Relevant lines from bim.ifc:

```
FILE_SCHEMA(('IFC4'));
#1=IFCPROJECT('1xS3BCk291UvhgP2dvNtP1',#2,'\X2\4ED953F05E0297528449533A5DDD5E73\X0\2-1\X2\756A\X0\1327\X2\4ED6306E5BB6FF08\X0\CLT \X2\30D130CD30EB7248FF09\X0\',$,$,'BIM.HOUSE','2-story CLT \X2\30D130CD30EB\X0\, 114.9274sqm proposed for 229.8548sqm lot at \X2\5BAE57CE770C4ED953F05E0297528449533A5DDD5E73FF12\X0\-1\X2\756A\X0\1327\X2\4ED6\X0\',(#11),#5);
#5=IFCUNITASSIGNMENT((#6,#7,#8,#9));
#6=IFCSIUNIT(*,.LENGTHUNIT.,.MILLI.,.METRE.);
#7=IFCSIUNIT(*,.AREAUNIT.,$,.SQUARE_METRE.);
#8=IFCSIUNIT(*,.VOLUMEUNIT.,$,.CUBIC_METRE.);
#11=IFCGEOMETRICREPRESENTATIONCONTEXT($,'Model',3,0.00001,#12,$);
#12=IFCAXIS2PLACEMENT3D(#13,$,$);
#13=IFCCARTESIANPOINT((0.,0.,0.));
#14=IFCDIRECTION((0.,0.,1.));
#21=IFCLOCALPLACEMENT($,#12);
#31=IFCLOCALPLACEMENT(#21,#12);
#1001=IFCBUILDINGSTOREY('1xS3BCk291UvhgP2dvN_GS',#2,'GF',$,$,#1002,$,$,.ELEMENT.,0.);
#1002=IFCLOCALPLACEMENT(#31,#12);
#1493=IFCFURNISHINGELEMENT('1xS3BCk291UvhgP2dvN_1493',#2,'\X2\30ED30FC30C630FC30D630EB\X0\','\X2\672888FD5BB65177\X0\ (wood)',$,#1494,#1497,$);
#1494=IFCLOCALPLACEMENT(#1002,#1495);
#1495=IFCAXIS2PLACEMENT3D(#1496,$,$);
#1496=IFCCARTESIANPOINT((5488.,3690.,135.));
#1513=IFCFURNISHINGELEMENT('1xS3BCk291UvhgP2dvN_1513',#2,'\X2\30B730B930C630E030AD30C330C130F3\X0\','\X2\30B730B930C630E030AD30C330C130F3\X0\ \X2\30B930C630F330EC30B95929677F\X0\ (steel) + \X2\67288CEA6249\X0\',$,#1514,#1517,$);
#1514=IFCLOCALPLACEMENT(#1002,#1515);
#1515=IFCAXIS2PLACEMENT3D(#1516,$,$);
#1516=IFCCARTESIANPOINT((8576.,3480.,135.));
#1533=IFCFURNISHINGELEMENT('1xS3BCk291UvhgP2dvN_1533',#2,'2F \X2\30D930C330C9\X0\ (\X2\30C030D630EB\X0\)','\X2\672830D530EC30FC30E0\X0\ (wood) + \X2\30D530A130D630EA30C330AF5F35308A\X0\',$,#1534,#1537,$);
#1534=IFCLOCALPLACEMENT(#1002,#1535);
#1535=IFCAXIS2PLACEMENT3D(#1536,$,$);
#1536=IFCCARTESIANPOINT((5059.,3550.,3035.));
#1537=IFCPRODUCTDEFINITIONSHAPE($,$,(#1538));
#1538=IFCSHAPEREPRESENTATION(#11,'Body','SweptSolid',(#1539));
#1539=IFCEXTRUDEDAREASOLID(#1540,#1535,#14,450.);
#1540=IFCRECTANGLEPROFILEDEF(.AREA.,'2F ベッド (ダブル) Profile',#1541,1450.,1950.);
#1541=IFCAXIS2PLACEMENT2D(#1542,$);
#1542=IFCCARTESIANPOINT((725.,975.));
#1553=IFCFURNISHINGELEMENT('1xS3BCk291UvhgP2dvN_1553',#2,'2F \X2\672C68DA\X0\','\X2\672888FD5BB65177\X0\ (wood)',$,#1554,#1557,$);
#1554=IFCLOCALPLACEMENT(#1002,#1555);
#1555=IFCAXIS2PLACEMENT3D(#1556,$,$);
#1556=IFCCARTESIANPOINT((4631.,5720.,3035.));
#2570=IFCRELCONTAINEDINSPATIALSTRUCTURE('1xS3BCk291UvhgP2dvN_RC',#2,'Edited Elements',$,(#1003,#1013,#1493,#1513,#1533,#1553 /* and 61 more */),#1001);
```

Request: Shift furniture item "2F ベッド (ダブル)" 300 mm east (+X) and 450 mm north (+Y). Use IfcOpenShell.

```python
import ifcopenshell
import ifcopenshell.api.geometry
import ifcopenshell.util.placement
import ifcopenshell.util.unit

model = ifcopenshell.open("bim.ifc")
unit_scale = ifcopenshell.util.unit.calculate_unit_scale(model)

item = model.by_id(1533)
matrix = ifcopenshell.util.placement.get_local_placement(item.ObjectPlacement)
matrix[0, 3] += 0.3 / unit_scale
matrix[1, 3] += 0.45 / unit_scale
ifcopenshell.api.geometry.edit_object_placement(model, product=item, matrix=matrix, is_si=False)

print(ifcopenshell.util.placement.get_local_placement(item.ObjectPlacement).round(3) + 0.0)

model.write("bim_v2.ifc")
```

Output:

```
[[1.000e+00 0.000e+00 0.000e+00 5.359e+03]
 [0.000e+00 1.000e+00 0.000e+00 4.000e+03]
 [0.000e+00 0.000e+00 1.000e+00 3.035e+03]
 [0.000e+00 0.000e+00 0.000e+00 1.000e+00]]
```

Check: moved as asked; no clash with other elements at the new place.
